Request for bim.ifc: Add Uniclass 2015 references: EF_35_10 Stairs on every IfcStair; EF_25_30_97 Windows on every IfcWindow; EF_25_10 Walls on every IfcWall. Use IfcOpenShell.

First a look at what the model holds.

```python
import ifcopenshell

model = ifcopenshell.open("bim.ifc")
print(model.schema)
print("classifications:", [c.Name for c in model.by_type("IfcClassification")])
for ifc_class in ("IfcDoor", "IfcRoof", "IfcStair", "IfcWall", "IfcWindow"):
    print(ifc_class, len(model.by_type(ifc_class)))
```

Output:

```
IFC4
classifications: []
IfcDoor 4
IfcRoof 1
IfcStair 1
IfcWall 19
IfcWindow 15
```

```python
import ifcopenshell
import ifcopenshell.api.classification

model = ifcopenshell.open("bim.ifc")

system = ifcopenshell.api.classification.add_classification(model, classification="Uniclass 2015")

codes = {
    "IfcStair": ("EF_35_10", "Stairs"),
    "IfcWindow": ("EF_25_30_97", "Windows"),
    "IfcWall": ("EF_25_10", "Walls"),
}
for ifc_class, (code, name) in codes.items():
    products = model.by_type(ifc_class)
    ifcopenshell.api.classification.add_reference(
        model, products=products, classification=system, identification=code, name=name
    )
    print(code, len(products))

model.write("bim-out.ifc")
```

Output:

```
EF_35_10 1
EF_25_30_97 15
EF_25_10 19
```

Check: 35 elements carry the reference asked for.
